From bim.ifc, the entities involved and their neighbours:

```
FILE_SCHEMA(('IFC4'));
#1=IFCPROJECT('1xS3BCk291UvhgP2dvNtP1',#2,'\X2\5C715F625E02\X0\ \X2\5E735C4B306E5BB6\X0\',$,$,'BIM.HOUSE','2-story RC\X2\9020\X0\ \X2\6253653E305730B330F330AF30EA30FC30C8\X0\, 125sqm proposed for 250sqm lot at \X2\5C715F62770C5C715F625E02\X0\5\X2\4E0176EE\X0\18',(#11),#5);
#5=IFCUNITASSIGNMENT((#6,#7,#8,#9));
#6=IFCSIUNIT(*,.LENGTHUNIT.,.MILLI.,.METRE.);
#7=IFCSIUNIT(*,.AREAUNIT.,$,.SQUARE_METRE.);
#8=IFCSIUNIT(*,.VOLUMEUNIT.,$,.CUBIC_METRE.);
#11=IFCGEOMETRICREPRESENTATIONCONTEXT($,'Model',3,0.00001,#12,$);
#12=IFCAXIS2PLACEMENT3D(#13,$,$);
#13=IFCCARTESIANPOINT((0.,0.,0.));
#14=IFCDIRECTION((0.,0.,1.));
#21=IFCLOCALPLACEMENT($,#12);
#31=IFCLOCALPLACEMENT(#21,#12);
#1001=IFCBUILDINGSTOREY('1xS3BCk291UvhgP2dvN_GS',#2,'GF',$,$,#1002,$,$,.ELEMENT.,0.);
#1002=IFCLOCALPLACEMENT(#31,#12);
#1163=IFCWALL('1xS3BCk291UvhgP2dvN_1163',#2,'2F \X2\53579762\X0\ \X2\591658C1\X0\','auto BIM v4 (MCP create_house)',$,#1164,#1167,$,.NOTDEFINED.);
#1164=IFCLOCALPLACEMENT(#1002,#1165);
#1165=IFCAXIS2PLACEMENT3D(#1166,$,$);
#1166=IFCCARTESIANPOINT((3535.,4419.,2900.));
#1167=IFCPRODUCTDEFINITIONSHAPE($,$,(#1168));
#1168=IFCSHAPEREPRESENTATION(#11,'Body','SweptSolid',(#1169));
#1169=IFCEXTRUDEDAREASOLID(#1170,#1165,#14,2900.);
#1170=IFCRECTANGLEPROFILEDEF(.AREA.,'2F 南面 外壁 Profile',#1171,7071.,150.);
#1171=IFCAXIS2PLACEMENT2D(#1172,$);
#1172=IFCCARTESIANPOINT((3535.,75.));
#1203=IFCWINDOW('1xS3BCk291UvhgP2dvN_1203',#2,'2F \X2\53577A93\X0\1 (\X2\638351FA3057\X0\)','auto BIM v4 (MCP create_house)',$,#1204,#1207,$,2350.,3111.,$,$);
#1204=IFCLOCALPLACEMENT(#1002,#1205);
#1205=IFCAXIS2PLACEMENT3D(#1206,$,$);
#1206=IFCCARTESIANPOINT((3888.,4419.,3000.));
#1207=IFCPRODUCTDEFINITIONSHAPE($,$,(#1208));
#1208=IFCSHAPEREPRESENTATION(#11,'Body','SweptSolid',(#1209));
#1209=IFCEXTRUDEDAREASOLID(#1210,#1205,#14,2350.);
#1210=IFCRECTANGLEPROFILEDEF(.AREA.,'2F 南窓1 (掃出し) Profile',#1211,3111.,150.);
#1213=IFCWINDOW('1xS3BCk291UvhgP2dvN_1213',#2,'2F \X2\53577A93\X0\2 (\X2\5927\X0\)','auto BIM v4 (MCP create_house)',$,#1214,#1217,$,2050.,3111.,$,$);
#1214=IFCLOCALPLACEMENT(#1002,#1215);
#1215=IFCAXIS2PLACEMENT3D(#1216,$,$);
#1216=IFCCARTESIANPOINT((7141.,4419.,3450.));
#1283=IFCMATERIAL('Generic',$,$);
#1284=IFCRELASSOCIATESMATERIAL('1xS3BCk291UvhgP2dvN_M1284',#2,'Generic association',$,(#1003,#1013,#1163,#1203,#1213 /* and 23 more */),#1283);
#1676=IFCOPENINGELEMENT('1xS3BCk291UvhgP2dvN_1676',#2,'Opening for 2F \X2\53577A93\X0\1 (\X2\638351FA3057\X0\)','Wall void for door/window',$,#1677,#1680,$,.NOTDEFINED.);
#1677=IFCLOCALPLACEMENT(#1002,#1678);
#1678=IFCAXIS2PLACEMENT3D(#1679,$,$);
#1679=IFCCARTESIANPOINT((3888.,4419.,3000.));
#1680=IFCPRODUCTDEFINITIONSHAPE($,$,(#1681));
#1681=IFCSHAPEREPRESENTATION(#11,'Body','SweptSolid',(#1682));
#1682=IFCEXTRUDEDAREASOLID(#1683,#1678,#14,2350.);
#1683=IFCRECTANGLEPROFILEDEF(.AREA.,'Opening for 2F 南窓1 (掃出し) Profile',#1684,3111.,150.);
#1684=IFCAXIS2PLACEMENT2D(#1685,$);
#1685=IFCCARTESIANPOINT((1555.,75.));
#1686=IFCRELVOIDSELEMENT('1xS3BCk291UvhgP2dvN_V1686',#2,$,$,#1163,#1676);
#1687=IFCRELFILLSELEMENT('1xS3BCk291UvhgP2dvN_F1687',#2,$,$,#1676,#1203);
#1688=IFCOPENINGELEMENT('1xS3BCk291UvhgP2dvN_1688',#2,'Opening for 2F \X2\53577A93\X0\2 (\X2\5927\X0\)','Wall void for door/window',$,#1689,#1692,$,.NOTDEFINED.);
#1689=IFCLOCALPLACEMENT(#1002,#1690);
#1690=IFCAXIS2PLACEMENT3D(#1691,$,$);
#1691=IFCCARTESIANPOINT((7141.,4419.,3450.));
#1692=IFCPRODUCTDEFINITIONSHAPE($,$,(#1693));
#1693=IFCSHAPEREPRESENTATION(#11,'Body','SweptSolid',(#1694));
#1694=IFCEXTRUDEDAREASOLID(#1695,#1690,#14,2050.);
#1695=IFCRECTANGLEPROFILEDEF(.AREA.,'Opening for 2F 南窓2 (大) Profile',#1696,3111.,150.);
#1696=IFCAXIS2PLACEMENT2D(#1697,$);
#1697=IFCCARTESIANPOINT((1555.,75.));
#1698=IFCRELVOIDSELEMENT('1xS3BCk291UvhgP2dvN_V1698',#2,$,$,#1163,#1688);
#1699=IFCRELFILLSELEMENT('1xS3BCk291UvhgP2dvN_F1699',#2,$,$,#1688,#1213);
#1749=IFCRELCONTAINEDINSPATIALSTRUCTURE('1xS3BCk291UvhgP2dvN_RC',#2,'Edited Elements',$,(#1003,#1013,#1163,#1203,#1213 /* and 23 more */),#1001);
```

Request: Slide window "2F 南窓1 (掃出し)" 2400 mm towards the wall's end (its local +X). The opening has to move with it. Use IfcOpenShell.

```python
import ifcopenshell
import ifcopenshell.api.geometry
import ifcopenshell.util.placement
import ifcopenshell.util.unit

model = ifcopenshell.open("bim.ifc")
unit_scale = ifcopenshell.util.unit.calculate_unit_scale(model)

window = model.by_id(1203)
opening = window.FillsVoids[0].RelatingOpeningElement
wall = opening.VoidsElements[0].RelatingBuildingElement

wall_matrix = ifcopenshell.util.placement.get_local_placement(wall.ObjectPlacement)
shift = wall_matrix[:3, 0] * 2.4 / unit_scale
before = ifcopenshell.util.placement.get_local_placement(window.ObjectPlacement)[:3, 3].copy()

# The window is not placed relative to its opening, so move both.
for product in (opening, window):
    matrix = ifcopenshell.util.placement.get_local_placement(product.ObjectPlacement)
    matrix[:3, 3] += shift
    ifcopenshell.api.geometry.edit_object_placement(model, product=product, matrix=matrix, is_si=False)

after = ifcopenshell.util.placement.get_local_placement(window.ObjectPlacement)[:3, 3]
print("window moved by", (after - before).round(3) + 0.0)

model.write("bim_edited.ifc")
```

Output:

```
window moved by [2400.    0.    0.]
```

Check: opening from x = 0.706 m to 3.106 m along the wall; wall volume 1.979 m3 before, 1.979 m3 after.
